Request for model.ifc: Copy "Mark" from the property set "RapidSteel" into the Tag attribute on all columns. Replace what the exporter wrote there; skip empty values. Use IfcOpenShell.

First a look at what the model holds.

```python
import ifcopenshell
import ifcopenshell.util.element

model = ifcopenshell.open("model.ifc")
print(model.schema)
columns = model.by_type("IfcColumn")
print(len(columns), "columns")
for e in columns[:8]:
    source = ifcopenshell.util.element.get_pset(e, "RapidSteel", "Mark")
    target = e.Tag
    print(e.id(), repr(source), repr(target), sep=" | ")
```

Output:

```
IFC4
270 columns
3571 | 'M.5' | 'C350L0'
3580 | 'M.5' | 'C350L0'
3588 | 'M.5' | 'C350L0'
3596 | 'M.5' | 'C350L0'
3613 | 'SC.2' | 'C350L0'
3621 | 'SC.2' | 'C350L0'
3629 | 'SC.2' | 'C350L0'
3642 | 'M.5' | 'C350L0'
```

```python
import ifcopenshell
import ifcopenshell.util.element

model = ifcopenshell.open("model.ifc")

count = 0
for e in model.by_type("IfcColumn"):
    value = ifcopenshell.util.element.get_pset(e, "RapidSteel", "Mark")
    current = e.Tag
    if not value or not value.strip() or current == value:
        continue
    e.Tag = value
    count += 1

print(count, "columns updated")

model.write("model_v2.ifc")
```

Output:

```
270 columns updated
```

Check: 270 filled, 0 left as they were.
